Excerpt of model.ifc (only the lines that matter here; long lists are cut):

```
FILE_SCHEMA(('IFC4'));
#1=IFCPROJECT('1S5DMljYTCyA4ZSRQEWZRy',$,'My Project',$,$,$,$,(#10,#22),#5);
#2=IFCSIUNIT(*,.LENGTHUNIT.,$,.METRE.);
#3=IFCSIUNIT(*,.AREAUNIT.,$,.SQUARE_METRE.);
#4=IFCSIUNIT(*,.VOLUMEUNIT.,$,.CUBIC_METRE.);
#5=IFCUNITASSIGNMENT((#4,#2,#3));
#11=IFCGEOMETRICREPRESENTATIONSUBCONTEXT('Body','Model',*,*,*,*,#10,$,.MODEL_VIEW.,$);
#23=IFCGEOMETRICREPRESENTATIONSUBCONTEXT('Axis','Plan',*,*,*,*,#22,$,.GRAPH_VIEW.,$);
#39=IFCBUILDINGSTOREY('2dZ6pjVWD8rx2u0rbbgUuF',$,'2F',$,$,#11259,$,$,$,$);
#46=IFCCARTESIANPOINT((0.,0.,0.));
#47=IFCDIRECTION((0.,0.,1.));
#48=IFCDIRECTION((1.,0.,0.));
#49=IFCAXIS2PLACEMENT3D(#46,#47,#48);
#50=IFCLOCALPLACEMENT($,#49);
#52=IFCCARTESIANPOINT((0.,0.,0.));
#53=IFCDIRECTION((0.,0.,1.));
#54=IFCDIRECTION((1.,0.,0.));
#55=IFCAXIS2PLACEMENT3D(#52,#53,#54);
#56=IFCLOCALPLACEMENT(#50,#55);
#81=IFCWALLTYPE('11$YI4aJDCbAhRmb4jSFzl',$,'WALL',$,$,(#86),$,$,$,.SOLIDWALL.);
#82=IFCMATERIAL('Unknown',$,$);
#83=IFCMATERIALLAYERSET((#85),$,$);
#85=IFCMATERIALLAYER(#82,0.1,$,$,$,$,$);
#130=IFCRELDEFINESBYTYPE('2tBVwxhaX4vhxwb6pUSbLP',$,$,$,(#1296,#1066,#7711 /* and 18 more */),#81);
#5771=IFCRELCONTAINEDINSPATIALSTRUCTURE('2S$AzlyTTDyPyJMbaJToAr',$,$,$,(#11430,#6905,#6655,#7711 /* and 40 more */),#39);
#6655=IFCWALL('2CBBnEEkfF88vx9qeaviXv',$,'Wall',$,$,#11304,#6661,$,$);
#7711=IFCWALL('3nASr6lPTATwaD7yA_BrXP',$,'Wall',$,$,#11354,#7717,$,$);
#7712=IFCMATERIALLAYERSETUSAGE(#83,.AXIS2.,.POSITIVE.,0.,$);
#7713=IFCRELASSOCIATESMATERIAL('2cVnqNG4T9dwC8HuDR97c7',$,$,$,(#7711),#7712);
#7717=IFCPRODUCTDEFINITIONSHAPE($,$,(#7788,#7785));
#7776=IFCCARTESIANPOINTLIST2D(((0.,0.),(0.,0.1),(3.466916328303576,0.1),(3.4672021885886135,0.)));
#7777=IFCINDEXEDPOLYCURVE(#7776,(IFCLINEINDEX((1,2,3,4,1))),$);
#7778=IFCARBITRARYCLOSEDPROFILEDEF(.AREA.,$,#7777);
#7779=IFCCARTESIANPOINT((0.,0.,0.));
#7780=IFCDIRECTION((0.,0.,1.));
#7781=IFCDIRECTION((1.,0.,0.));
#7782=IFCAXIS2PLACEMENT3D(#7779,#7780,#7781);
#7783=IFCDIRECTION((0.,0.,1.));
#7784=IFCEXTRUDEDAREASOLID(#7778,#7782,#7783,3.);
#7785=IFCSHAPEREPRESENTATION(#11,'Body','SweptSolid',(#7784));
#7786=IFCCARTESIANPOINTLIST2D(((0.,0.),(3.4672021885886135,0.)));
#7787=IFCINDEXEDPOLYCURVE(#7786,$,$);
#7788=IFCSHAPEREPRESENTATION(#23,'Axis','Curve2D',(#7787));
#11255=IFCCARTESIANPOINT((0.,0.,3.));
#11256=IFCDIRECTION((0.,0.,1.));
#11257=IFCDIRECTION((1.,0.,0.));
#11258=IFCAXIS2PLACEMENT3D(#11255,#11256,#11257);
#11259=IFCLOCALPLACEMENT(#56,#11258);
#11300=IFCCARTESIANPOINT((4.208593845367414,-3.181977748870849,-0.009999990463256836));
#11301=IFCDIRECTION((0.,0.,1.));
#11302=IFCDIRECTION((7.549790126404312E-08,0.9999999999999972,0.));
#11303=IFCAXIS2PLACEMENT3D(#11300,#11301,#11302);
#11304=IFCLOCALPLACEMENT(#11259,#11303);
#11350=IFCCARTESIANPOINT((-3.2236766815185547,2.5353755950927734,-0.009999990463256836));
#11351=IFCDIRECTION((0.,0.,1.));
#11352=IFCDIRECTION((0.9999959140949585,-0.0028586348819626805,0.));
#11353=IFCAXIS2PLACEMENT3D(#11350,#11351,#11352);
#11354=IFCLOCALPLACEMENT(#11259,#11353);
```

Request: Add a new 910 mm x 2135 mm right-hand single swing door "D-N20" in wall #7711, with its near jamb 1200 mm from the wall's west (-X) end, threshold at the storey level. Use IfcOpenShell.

```python
import numpy as np
import ifcopenshell
import ifcopenshell.api.feature
import ifcopenshell.api.geometry
import ifcopenshell.api.root
import ifcopenshell.api.spatial
import ifcopenshell.geom
import ifcopenshell.util.element
import ifcopenshell.util.placement
import ifcopenshell.util.representation
import ifcopenshell.util.shape
import ifcopenshell.util.unit

model = ifcopenshell.open("model.ifc")
unit_scale = ifcopenshell.util.unit.calculate_unit_scale(model)
settings = ifcopenshell.geom.settings()


def volume(element):
    """Net volume in cubic metres, openings subtracted."""
    shape = ifcopenshell.geom.create_shape(settings, element)
    return ifcopenshell.util.shape.get_volume(shape.geometry)


wall = model.by_id(7711)
storey = ifcopenshell.util.element.get_container(wall, ifc_class="IfcBuildingStorey")
context = ifcopenshell.util.representation.get_context(model, "Model", "Body", "MODEL_VIEW")
before = volume(wall)

width, height, from_end, sill = 0.91, 2.135, 1.2, 0.0  # metres

# The wall runs along its own X axis, and the end named is its -X end.
wall_shape = ifcopenshell.geom.create_shape(settings, wall)
x, y, z = ifcopenshell.util.shape.get_vertices(wall_shape.geometry).T
start = x.min() + from_end
face, thickness = float(y.min()), float(y.max() - y.min())
wall_matrix = ifcopenshell.util.placement.get_local_placement(wall.ObjectPlacement)
level = ifcopenshell.util.placement.get_local_placement(storey.ObjectPlacement)[2, 3]


def in_wall(x, y):
    """Placement at x, y metres in the wall's axes, at sill height."""
    matrix = wall_matrix.copy()
    matrix[:, 3] = wall_matrix @ np.array([x / unit_scale, y / unit_scale, 0.0, 1.0])
    matrix[2, 3] = level + sill / unit_scale
    return matrix


# Opening: a box that overshoots both wall faces by 50 mm.
opening = ifcopenshell.api.root.create_entity(model, ifc_class="IfcOpeningElement", predefined_type="OPENING")
box = ifcopenshell.api.geometry.add_wall_representation(
    model, context=context, length=width, height=height, thickness=thickness + 0.1
)
ifcopenshell.api.geometry.assign_representation(model, product=opening, representation=box)
ifcopenshell.api.geometry.edit_object_placement(model, product=opening, matrix=in_wall(start, face - 0.05), is_si=False)
ifcopenshell.api.feature.add_feature(model, feature=opening, element=wall)

door = ifcopenshell.api.root.create_entity(model, ifc_class="IfcDoor", name="D-N20", predefined_type="DOOR")
door.OverallWidth, door.OverallHeight = width / unit_scale, height / unit_scale
door.OperationType = "SINGLE_SWING_RIGHT"
body = ifcopenshell.api.geometry.add_door_representation(
    model,
    context=context,
    overall_width=door.OverallWidth,
    overall_height=door.OverallHeight,
    operation_type="SINGLE_SWING_RIGHT",
    lining_properties={"LiningDepth": thickness / unit_scale, "ThresholdDepth": thickness / unit_scale},
)
ifcopenshell.api.geometry.assign_representation(model, product=door, representation=body)
ifcopenshell.api.spatial.assign_container(model, products=[door], relating_structure=storey)
ifcopenshell.api.feature.add_filling(model, opening=opening, element=door)

# The lining spans the wall, so the door starts at the wall face.
ifcopenshell.api.geometry.edit_object_placement(model, product=door, matrix=in_wall(start, face), is_si=False)

after = volume(wall)

print(f"wall volume {before:.3f} -> {after:.3f} m3")

model.write("model_edited.ifc")
```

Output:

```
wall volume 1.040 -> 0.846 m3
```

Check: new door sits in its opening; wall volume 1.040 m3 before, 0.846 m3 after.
